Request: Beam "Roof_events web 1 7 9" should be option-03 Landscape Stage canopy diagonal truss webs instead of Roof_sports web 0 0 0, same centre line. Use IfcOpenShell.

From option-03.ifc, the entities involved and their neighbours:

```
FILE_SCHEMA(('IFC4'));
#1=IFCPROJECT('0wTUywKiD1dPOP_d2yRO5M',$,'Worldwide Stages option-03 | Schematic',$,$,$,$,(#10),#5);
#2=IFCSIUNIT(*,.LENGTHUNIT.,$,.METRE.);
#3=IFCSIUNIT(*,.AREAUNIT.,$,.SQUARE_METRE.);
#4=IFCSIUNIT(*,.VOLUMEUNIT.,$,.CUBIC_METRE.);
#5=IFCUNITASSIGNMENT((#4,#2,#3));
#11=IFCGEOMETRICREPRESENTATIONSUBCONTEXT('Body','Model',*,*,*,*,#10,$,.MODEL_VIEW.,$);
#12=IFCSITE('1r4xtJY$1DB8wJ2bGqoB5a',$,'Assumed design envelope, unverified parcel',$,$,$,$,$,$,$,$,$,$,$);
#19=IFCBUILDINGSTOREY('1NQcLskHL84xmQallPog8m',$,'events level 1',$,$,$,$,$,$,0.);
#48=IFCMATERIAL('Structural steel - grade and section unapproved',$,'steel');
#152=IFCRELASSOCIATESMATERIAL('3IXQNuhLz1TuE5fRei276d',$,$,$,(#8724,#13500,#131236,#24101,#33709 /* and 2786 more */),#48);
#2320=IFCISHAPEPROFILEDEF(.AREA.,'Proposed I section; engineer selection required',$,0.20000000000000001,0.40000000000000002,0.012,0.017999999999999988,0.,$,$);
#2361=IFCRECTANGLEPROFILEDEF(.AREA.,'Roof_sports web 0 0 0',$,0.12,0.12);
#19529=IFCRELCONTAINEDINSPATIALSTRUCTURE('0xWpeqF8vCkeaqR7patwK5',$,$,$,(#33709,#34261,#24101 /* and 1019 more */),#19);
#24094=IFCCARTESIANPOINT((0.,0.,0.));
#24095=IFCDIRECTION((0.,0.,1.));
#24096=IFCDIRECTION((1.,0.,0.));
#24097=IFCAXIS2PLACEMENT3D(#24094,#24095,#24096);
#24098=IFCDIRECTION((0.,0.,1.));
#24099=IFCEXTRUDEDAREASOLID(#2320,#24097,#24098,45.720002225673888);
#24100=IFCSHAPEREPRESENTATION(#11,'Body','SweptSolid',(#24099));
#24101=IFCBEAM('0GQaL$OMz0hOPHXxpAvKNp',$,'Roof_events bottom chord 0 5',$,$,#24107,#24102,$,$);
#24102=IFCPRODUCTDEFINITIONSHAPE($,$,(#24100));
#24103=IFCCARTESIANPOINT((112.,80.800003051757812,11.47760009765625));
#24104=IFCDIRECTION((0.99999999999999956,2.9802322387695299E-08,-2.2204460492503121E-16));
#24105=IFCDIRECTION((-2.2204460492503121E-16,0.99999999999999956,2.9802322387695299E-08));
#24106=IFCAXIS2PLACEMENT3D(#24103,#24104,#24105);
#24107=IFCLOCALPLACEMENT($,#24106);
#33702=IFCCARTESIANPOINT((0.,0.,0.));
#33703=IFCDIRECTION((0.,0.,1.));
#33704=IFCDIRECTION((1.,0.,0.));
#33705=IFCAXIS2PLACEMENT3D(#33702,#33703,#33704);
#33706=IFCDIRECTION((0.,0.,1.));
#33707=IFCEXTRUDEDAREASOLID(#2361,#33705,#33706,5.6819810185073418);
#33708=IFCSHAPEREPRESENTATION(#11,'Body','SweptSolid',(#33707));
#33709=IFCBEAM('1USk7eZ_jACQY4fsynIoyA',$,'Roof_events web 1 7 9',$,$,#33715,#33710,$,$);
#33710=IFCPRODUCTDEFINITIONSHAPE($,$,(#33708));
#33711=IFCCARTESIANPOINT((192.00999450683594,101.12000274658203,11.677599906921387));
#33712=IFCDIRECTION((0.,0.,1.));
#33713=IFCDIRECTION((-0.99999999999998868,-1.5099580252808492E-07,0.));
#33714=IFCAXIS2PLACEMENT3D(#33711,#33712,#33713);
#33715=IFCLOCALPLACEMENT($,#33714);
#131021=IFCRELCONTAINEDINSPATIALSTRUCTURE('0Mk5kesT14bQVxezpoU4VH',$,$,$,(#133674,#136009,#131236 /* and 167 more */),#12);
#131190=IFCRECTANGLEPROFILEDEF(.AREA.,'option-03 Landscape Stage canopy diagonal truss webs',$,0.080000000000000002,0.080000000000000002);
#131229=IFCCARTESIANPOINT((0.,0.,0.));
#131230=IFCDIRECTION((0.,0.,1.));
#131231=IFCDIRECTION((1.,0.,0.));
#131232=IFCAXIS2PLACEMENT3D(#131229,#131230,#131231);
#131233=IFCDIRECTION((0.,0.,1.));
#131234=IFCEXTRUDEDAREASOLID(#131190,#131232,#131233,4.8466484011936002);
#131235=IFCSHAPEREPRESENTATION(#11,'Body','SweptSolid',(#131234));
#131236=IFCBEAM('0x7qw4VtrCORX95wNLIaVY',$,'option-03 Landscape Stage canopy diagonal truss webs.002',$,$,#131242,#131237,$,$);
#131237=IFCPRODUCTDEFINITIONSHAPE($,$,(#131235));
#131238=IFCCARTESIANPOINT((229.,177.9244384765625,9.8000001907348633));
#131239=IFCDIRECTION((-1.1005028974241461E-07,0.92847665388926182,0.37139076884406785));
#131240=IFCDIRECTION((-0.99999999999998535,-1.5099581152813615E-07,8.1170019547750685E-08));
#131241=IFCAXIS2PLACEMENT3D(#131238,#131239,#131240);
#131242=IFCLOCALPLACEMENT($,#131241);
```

```python
import ifcopenshell
import ifcopenshell.util.element
import ifcopenshell.util.representation

model = ifcopenshell.open("option-03.ifc")

member = model.by_id(33709)
source = next(p for p in model.by_type("IfcRectangleProfileDef") if p.ProfileName == "option-03 Landscape Stage canopy diagonal truss webs")

body = ifcopenshell.util.representation.get_representation(member, "Model", "Body")
solid = body.Items[0]
old_profile = solid.SweptArea

# Copy the section's sizes but keep this member's own profile position.
profile = ifcopenshell.util.element.copy(model, source)
profile.Position = old_profile.Position
solid.SweptArea = profile
if not model.get_total_inverses(old_profile):
    ifcopenshell.util.element.remove_deep2(model, old_profile)

print(solid.SweptArea)

model.write("option-03_v2.ifc")
```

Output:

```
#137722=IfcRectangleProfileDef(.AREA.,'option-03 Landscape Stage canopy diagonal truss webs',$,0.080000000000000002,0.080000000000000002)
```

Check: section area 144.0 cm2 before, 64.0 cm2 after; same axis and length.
